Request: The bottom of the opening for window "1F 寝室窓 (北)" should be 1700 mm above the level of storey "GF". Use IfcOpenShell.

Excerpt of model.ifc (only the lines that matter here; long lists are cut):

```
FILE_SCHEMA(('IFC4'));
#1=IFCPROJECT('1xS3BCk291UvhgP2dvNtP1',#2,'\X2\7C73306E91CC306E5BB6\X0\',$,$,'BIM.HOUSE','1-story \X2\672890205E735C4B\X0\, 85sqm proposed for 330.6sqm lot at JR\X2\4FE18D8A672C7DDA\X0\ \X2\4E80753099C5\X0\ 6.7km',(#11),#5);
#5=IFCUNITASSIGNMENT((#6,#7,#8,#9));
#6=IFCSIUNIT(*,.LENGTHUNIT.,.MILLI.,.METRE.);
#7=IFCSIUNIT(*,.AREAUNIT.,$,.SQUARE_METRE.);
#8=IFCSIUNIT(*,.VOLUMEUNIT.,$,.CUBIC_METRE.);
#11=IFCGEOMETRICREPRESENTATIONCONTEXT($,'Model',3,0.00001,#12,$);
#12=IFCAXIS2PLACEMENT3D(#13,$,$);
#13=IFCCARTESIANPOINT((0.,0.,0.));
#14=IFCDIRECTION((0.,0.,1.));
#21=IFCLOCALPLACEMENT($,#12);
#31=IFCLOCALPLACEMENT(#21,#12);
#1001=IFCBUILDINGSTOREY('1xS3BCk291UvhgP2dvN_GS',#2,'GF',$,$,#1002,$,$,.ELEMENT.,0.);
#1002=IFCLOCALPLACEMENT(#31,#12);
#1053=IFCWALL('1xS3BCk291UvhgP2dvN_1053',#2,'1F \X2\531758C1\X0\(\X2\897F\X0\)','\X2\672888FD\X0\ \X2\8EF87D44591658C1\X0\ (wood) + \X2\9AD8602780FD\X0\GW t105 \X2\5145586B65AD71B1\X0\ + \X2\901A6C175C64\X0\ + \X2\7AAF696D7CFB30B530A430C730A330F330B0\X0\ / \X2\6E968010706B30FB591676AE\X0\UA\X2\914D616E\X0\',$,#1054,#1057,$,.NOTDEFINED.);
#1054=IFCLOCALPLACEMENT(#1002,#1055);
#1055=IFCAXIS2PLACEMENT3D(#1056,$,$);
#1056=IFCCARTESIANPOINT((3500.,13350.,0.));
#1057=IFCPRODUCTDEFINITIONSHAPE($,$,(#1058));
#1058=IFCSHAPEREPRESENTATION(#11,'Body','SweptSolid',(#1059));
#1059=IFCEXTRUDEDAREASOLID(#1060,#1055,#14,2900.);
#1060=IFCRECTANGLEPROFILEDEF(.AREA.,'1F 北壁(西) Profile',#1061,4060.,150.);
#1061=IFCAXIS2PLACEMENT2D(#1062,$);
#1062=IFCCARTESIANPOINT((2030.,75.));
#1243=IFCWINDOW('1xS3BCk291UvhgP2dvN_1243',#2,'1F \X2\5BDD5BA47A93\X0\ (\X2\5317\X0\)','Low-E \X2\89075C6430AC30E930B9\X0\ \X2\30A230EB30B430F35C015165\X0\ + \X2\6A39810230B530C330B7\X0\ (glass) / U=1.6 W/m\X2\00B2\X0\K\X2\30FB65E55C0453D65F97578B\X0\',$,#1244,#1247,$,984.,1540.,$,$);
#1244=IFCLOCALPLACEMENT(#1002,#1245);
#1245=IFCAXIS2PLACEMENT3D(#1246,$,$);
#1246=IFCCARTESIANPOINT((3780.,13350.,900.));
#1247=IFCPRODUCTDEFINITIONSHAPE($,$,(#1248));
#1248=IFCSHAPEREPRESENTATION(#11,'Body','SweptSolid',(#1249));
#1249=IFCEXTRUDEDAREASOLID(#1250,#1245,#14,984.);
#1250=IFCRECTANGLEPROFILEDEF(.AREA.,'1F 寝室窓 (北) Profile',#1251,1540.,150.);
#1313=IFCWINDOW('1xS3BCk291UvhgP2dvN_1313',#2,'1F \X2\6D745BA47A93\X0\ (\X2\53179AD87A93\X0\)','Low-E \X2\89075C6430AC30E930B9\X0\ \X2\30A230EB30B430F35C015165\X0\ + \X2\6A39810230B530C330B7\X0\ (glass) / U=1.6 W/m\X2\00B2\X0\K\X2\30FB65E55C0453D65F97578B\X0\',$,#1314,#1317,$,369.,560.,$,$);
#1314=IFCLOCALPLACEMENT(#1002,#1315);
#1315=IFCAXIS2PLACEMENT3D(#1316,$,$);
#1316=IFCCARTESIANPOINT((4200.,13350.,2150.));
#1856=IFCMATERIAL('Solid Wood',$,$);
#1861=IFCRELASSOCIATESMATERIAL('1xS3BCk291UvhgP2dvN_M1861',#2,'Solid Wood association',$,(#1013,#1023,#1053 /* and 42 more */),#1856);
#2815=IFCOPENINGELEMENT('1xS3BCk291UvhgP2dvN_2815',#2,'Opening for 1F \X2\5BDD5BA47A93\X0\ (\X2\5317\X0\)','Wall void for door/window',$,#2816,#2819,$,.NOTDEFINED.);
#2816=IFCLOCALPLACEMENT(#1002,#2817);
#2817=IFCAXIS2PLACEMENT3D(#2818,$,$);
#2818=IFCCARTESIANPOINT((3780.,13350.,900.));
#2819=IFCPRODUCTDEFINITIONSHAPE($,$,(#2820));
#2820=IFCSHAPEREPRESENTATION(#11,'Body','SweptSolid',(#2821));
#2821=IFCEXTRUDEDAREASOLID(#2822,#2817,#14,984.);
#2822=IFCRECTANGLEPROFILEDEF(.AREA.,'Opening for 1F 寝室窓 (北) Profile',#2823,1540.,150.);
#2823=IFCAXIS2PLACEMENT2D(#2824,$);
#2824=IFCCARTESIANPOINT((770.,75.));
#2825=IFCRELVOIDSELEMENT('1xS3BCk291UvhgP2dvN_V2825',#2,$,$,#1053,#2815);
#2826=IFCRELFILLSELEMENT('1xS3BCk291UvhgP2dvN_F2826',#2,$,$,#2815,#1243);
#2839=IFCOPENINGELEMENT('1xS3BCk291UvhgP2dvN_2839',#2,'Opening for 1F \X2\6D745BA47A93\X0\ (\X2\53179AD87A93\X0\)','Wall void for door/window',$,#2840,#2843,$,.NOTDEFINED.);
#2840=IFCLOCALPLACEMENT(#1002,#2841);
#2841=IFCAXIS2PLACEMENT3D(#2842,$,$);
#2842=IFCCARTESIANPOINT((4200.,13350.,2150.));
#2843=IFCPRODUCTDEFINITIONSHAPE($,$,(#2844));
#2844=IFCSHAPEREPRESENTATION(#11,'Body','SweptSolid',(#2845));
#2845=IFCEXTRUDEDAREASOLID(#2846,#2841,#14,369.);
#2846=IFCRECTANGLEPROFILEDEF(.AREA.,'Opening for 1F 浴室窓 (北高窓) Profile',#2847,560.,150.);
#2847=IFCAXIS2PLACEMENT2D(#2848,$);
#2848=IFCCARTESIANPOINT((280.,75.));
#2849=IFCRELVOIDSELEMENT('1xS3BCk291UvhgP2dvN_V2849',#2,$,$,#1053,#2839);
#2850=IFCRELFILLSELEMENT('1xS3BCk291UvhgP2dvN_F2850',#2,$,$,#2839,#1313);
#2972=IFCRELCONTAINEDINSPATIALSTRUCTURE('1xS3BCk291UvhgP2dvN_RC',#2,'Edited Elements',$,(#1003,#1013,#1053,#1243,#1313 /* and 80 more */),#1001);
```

```python
import numpy as np
import ifcopenshell
import ifcopenshell.api.geometry
import ifcopenshell.geom
import ifcopenshell.util.element
import ifcopenshell.util.placement
import ifcopenshell.util.shape
import ifcopenshell.util.unit

model = ifcopenshell.open("model.ifc")
unit_scale = ifcopenshell.util.unit.calculate_unit_scale(model)

window = model.by_guid("1xS3BCk291UvhgP2dvN_1243")
opening = window.FillsVoids[0].RelatingOpeningElement
storey = ifcopenshell.util.element.get_container(window, ifc_class="IfcBuildingStorey")
level = ifcopenshell.util.placement.get_local_placement(storey.ObjectPlacement)[2, 3]

# The opening's origin need not be at the sill, so measure its lowest point.
shape = ifcopenshell.geom.create_shape(ifcopenshell.geom.settings(), opening)
bottom = ifcopenshell.util.shape.get_shape_bottom_elevation(shape, shape.geometry) / unit_scale
dz = level + 1700.0 - bottom

shift = np.array([0.0, 0.0, dz])
# The window is not placed relative to its opening, so move both.
for product in (opening, window):
    matrix = ifcopenshell.util.placement.get_local_placement(product.ObjectPlacement)
    matrix[:3, 3] += shift
    ifcopenshell.api.geometry.edit_object_placement(model, product=product, matrix=matrix, is_si=False)

print(f"moved by {dz * unit_scale:+.3f} m")

model.write("model_rev.ifc")
```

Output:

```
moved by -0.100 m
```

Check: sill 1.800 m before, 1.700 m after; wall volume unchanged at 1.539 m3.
